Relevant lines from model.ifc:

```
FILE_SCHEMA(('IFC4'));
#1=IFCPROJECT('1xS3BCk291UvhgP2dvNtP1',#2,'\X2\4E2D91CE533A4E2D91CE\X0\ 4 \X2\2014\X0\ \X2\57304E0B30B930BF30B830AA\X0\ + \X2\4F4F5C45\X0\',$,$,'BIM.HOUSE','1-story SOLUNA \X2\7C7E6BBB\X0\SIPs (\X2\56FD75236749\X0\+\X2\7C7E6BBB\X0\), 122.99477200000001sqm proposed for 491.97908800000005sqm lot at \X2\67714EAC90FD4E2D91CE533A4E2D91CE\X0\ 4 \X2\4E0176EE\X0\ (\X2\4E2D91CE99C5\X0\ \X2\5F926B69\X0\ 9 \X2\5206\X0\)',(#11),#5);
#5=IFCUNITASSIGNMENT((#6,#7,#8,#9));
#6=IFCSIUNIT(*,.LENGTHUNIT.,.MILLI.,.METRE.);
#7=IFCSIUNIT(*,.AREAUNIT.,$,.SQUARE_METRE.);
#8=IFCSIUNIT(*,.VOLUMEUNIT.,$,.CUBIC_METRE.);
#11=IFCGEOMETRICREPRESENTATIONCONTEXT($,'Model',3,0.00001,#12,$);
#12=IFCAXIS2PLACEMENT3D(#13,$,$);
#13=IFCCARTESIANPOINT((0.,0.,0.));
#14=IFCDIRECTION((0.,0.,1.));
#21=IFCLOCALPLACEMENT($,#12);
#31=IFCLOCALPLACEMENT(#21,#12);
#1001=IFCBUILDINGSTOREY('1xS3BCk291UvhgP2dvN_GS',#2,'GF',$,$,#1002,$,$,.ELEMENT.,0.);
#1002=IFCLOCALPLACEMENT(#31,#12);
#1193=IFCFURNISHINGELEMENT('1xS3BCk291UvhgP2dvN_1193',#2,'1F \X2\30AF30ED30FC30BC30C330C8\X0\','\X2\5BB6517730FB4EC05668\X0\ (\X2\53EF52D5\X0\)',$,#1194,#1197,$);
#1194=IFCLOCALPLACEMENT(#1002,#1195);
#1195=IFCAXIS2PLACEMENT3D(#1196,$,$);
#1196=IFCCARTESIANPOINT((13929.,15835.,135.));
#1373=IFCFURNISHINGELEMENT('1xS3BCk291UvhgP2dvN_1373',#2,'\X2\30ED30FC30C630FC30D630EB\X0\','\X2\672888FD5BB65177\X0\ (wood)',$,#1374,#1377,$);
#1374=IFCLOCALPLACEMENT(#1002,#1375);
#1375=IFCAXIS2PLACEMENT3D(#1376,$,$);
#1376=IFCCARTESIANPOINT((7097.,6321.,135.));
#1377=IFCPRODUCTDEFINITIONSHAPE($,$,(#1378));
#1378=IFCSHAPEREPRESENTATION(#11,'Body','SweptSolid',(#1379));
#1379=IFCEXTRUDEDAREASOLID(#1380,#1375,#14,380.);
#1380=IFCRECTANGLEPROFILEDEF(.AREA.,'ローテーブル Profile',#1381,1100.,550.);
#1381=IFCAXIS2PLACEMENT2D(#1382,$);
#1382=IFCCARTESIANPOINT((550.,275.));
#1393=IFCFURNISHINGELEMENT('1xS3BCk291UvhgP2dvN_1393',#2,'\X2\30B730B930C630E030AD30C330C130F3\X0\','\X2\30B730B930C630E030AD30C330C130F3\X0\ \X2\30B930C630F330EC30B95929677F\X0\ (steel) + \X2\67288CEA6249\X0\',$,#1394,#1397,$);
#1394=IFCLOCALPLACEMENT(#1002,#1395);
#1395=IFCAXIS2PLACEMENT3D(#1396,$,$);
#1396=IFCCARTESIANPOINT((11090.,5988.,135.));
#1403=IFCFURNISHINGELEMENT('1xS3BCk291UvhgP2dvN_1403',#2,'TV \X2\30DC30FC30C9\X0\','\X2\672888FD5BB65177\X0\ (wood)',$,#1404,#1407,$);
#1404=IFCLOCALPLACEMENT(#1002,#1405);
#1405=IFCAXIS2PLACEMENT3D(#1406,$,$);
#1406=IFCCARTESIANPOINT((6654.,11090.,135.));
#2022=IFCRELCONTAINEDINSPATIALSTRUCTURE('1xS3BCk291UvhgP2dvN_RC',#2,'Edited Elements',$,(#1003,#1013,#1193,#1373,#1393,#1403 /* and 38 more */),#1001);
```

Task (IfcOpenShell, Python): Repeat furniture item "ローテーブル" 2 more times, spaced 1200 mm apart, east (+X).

```python
import numpy as np
import ifcopenshell
import ifcopenshell.api.geometry
import ifcopenshell.api.root
import ifcopenshell.util.element
import ifcopenshell.util.placement

model = ifcopenshell.open("model.ifc")


def reuse_history(source, copy):
    """copy_class also copies each property set's owner history, people and application; keep the originals."""
    for rel in copy.IsDefinedBy:
        if rel.is_a("IfcRelDefinesByProperties") and (history := rel.RelatingPropertyDefinition.OwnerHistory):
            rel.RelatingPropertyDefinition.OwnerHistory = source.OwnerHistory
            ifcopenshell.util.element.remove_deep2(model, history)


source = model.by_guid("1xS3BCk291UvhgP2dvN_1373")
base = ifcopenshell.util.placement.get_local_placement(source.ObjectPlacement)
step = np.array([1.0, 0.0, 0.0]) * 1200.0

for i in range(1, 3):
    copy = ifcopenshell.api.root.copy_class(model, product=source)
    copy.Representation = ifcopenshell.util.element.copy_deep(
        model, source.Representation, exclude=["IfcGeometricRepresentationContext", "IfcRepresentationMap"]
    )
    reuse_history(source, copy)
    matrix = base.copy()
    matrix[:3, 3] += i * step
    print("added at", matrix[:3, 3].round(3) + 0.0)
    ifcopenshell.api.geometry.edit_object_placement(model, product=copy, matrix=matrix, is_si=False)

model.write("model_updated.ifc")
```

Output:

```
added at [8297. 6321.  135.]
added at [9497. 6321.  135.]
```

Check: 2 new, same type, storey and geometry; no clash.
